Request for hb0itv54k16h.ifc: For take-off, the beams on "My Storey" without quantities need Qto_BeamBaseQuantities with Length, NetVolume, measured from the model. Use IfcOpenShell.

First a look at what the model holds.

```python
import ifcopenshell
import ifcopenshell.util.element
import ifcopenshell.util.unit

model = ifcopenshell.open("hb0itv54k16h.ifc")
print(model.schema)
for unit_type in ("LENGTHUNIT", "AREAUNIT", "VOLUMEUNIT"):
    print(unit_type, ifcopenshell.util.unit.calculate_unit_scale(model, unit_type))
storey = next(s for s in model.by_type("IfcBuildingStorey") if s.Name == "My Storey")
beams = [e for e in ifcopenshell.util.element.get_decomposition(storey) if e.is_a("IfcBeam")]
for e in sorted(beams, key=lambda e: e.id()):
    print(e.id(), e.is_a(), e.Name, list(ifcopenshell.util.element.get_psets(e, qtos_only=True)), sep=" | ")
```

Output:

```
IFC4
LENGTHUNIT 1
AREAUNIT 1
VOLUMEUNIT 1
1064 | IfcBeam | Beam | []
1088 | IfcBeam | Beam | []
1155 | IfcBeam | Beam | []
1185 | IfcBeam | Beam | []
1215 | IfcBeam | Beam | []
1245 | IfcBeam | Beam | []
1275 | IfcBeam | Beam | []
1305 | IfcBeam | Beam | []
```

```python
import ifcopenshell
import ifcopenshell.api.pset
import ifcopenshell.geom
import ifcopenshell.util.element
import ifcopenshell.util.shape
import ifcopenshell.util.unit

model = ifcopenshell.open("hb0itv54k16h.ifc")
unit_scale = ifcopenshell.util.unit.calculate_unit_scale(model)
volume_scale = ifcopenshell.util.unit.calculate_unit_scale(model, "VOLUMEUNIT")
settings = ifcopenshell.geom.settings()

storey = next(s for s in model.by_type("IfcBuildingStorey") if s.Name == "My Storey")
beams = [e for e in ifcopenshell.util.element.get_decomposition(storey) if e.is_a("IfcBeam")]

for e in sorted(beams, key=lambda e: e.id()):
    if ifcopenshell.util.element.get_psets(e, qtos_only=True, should_inherit=False):
        continue
    # Geometry comes back in metres, in the element's own axes.
    shape = ifcopenshell.geom.create_shape(settings, e)
    values = {
        "Length": ifcopenshell.util.shape.get_max_xyz(shape.geometry) / unit_scale,
        "NetVolume": ifcopenshell.util.shape.get_volume(shape.geometry) / volume_scale,
    }
    qto = ifcopenshell.api.pset.add_qto(model, product=e, name="Qto_BeamBaseQuantities")
    ifcopenshell.api.pset.edit_qto(model, qto=qto, properties=values)
    print(e.id(), {k: round(v, 3) for k, v in values.items()})

model.write("hb0itv54k16h_updated.ifc")
```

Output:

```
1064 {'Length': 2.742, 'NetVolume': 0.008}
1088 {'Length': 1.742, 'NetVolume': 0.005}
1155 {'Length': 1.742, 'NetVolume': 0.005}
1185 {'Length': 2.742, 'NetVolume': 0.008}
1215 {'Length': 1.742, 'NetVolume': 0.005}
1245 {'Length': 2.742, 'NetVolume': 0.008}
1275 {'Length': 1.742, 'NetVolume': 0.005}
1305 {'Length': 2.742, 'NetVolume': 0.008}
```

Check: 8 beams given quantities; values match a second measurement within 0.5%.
